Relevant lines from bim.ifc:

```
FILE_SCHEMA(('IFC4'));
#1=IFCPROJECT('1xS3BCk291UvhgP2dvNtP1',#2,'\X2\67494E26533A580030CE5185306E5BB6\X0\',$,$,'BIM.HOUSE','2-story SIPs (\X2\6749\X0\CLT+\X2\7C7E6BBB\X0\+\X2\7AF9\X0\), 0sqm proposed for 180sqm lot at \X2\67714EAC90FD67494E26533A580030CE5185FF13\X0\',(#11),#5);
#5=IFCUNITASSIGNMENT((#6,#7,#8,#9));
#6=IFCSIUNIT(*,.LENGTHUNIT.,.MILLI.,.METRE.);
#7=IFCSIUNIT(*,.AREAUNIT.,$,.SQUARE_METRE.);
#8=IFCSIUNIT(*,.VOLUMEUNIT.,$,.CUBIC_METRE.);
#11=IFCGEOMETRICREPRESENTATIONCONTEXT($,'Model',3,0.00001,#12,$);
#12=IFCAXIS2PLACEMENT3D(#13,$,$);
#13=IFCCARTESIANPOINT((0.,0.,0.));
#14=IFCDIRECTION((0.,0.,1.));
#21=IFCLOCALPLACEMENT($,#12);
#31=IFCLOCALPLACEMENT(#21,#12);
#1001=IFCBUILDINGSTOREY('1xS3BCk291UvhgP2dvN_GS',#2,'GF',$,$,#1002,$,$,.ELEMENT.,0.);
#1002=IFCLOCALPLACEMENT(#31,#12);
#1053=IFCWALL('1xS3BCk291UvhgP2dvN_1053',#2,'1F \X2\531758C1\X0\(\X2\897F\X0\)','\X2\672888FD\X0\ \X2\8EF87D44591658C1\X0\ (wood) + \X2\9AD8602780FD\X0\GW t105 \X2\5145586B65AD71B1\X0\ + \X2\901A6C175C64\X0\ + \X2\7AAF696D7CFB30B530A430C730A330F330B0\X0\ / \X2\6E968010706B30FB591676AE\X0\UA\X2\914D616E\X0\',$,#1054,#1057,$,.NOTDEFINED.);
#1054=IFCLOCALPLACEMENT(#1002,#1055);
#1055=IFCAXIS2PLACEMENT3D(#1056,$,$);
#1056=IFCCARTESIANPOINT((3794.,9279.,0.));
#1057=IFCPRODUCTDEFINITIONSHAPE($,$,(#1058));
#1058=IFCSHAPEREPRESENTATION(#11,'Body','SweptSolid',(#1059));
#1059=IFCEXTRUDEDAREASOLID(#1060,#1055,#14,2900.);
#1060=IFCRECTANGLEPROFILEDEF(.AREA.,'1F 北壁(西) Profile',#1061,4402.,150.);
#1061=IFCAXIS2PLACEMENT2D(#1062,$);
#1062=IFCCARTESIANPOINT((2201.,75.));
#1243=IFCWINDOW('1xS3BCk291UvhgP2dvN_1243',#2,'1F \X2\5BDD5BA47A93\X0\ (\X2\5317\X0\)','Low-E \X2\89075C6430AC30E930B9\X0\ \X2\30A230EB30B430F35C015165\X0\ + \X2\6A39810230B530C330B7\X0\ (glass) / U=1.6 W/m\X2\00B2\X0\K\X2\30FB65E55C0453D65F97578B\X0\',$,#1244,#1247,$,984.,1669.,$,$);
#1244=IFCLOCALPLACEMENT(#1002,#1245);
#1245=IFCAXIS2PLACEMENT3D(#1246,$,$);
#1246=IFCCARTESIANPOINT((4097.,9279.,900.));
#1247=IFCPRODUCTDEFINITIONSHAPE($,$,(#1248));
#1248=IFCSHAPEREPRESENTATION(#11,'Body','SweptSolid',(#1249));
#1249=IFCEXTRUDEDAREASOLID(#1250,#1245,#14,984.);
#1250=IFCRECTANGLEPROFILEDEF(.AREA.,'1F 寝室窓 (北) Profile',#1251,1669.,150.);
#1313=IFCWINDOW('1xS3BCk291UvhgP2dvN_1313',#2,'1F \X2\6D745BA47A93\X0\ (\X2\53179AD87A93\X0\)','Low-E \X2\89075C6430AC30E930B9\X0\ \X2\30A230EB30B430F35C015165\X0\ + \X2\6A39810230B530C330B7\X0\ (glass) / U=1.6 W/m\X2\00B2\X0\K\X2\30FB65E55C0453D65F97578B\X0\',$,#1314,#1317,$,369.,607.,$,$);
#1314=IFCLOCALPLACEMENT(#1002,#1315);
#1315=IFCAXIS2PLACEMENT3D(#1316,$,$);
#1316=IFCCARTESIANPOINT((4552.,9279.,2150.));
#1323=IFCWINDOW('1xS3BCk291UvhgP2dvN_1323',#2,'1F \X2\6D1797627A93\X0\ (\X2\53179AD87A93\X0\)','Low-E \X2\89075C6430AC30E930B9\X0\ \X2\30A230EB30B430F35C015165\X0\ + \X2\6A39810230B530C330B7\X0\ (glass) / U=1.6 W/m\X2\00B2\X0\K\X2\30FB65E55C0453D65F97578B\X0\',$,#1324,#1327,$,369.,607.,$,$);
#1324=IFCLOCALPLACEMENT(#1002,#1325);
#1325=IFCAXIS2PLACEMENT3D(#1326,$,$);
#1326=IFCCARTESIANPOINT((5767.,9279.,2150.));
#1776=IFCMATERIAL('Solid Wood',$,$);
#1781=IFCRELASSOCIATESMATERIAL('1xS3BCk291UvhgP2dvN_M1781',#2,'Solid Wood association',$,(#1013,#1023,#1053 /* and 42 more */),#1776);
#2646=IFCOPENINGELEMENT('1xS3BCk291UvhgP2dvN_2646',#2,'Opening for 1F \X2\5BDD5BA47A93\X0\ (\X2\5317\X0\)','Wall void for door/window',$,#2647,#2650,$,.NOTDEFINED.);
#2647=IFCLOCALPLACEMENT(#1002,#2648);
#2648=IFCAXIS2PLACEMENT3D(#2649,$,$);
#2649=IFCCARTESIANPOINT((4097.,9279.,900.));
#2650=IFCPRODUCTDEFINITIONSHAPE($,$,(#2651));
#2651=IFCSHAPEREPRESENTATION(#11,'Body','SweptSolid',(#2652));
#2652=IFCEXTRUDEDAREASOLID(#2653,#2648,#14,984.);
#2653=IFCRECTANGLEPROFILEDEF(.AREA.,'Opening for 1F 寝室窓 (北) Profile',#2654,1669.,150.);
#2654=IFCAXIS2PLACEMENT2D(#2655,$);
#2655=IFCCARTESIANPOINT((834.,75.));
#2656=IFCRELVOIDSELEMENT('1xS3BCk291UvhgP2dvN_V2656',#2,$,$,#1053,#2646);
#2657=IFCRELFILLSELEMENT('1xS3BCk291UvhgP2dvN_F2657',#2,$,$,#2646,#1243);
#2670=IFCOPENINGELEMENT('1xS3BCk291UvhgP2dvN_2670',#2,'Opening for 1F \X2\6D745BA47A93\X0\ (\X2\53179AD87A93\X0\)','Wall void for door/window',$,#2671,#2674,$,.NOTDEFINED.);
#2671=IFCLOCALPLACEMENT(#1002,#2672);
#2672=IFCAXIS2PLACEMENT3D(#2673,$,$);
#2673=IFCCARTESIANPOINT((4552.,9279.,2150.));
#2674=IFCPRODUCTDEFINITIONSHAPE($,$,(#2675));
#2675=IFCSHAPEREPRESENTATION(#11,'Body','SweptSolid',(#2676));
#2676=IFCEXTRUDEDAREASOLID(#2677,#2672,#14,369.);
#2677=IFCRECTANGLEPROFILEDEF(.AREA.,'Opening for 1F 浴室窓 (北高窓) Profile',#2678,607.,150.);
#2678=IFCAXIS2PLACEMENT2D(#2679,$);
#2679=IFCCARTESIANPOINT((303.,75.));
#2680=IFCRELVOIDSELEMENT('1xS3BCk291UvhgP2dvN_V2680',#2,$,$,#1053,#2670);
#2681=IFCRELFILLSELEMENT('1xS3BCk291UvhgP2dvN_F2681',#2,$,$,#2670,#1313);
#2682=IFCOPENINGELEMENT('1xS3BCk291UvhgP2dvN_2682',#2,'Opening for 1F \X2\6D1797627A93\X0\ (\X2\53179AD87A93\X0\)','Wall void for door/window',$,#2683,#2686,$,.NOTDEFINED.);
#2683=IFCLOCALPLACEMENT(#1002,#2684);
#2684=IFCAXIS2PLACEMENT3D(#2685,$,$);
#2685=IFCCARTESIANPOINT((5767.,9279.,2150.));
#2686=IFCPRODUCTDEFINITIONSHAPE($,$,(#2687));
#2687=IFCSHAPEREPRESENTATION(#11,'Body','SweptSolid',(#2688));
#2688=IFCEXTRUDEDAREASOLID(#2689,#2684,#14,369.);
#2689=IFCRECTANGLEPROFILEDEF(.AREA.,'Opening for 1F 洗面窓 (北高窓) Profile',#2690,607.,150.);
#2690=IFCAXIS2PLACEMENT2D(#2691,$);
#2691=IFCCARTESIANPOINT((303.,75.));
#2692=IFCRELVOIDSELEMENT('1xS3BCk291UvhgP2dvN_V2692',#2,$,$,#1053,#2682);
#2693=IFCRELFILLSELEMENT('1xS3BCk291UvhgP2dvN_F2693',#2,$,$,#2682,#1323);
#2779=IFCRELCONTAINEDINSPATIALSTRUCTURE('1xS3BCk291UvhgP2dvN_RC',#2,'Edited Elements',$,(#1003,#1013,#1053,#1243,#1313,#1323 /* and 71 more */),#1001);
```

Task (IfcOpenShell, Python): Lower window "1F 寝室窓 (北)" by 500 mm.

```python
import numpy as np
import ifcopenshell
import ifcopenshell.api.geometry
import ifcopenshell.util.placement
import ifcopenshell.util.unit

model = ifcopenshell.open("bim.ifc")
unit_scale = ifcopenshell.util.unit.calculate_unit_scale(model)

window = model.by_guid("1xS3BCk291UvhgP2dvN_1243")
opening = window.FillsVoids[0].RelatingOpeningElement
dz = -0.5 / unit_scale

shift = np.array([0.0, 0.0, dz])
# The window is not placed relative to its opening, so move both.
for product in (opening, window):
    matrix = ifcopenshell.util.placement.get_local_placement(product.ObjectPlacement)
    matrix[:3, 3] += shift
    ifcopenshell.api.geometry.edit_object_placement(model, product=product, matrix=matrix, is_si=False)

print(f"moved by {dz * unit_scale:+.3f} m")

model.write("bim_v2.ifc")
```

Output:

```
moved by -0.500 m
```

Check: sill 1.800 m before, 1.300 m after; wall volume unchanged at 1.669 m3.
